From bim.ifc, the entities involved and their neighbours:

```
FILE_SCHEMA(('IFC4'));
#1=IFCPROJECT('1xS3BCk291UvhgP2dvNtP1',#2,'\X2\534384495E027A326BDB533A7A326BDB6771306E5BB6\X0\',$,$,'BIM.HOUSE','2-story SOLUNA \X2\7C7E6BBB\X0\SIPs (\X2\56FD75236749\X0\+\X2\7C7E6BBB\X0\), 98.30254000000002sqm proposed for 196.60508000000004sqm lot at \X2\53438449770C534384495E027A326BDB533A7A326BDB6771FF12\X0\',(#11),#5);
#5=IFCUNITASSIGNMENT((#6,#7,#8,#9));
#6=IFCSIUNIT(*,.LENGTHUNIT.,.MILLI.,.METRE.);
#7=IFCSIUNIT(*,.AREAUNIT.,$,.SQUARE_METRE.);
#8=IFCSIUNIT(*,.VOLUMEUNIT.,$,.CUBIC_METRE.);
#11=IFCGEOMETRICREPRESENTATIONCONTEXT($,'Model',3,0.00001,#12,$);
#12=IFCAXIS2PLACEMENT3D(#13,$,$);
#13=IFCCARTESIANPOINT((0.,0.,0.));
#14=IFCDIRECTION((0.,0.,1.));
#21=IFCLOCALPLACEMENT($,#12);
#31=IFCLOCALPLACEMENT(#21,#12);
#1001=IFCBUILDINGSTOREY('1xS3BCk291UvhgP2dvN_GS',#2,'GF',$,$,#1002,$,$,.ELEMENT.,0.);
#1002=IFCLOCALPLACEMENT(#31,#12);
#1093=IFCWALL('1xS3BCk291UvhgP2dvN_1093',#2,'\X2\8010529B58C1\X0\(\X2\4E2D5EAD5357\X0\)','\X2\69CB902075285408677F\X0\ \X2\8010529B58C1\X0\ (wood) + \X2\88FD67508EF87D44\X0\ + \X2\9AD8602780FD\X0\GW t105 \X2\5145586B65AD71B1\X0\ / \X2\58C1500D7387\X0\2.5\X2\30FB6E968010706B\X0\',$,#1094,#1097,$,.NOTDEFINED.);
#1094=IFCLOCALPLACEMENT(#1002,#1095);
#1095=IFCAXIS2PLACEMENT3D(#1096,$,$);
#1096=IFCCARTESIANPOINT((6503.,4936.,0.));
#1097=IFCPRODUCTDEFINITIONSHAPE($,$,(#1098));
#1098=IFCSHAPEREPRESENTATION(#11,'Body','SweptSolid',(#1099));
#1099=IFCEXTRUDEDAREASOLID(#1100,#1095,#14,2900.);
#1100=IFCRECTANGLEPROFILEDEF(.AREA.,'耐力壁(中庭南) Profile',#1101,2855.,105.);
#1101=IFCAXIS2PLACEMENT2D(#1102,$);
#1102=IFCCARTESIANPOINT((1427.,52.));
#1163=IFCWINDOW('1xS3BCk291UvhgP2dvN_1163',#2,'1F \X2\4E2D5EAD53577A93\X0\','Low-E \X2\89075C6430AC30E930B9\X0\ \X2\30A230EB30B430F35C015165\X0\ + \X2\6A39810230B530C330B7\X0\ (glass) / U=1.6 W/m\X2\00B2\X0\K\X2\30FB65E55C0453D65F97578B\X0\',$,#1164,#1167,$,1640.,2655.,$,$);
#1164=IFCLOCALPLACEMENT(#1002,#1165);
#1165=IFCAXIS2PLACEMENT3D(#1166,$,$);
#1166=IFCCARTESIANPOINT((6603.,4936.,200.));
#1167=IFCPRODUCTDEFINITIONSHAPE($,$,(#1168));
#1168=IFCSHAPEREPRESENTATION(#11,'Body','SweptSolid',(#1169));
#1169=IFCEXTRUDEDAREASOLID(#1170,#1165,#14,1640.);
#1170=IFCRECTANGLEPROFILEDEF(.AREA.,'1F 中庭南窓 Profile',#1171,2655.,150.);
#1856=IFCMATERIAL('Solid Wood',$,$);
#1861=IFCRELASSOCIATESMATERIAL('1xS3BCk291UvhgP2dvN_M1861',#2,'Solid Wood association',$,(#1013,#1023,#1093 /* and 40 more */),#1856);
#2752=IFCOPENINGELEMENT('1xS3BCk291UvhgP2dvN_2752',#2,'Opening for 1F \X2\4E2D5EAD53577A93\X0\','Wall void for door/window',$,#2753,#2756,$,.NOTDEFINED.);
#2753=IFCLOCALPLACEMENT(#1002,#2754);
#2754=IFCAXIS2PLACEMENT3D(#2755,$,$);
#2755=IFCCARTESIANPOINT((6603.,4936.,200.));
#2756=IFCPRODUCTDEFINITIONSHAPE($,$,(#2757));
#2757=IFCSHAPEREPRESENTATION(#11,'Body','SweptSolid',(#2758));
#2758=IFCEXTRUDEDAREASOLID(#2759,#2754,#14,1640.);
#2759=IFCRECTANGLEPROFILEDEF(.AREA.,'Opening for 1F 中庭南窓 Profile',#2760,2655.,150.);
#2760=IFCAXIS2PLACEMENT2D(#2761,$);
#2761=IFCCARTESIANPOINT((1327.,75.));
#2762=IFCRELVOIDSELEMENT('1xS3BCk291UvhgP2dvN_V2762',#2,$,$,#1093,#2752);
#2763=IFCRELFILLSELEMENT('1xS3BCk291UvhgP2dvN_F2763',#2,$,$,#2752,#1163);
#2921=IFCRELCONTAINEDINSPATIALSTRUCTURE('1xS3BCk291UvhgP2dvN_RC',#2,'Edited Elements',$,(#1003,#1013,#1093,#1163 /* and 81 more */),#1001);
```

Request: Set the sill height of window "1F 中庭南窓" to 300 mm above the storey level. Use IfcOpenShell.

```python
import numpy as np
import ifcopenshell
import ifcopenshell.api.geometry
import ifcopenshell.geom
import ifcopenshell.util.element
import ifcopenshell.util.placement
import ifcopenshell.util.shape
import ifcopenshell.util.unit

model = ifcopenshell.open("bim.ifc")
unit_scale = ifcopenshell.util.unit.calculate_unit_scale(model)

window = model.by_guid("1xS3BCk291UvhgP2dvN_1163")
opening = window.FillsVoids[0].RelatingOpeningElement
storey = ifcopenshell.util.element.get_container(window, ifc_class="IfcBuildingStorey")
level = ifcopenshell.util.placement.get_local_placement(storey.ObjectPlacement)[2, 3]

# The opening's origin need not be at the sill, so measure its lowest point.
shape = ifcopenshell.geom.create_shape(ifcopenshell.geom.settings(), opening)
bottom = ifcopenshell.util.shape.get_shape_bottom_elevation(shape, shape.geometry) / unit_scale
dz = level + 0.3 / unit_scale - bottom

shift = np.array([0.0, 0.0, dz])
# The window is not placed relative to its opening, so move both.
for product in (opening, window):
    matrix = ifcopenshell.util.placement.get_local_placement(product.ObjectPlacement)
    matrix[:3, 3] += shift
    ifcopenshell.api.geometry.edit_object_placement(model, product=product, matrix=matrix, is_si=False)

print(f"moved by {dz * unit_scale:+.3f} m")

model.write("bim_v2.ifc")
```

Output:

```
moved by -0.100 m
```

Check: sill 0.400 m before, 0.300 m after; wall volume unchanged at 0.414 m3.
